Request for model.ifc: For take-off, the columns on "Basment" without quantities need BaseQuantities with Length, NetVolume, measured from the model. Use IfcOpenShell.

First a look at what the model holds.

```python
import ifcopenshell
import ifcopenshell.util.element
import ifcopenshell.util.unit

model = ifcopenshell.open("model.ifc")
print(model.schema)
for unit_type in ("LENGTHUNIT", "AREAUNIT", "VOLUMEUNIT"):
    print(unit_type, ifcopenshell.util.unit.calculate_unit_scale(model, unit_type))
storey = next(s for s in model.by_type("IfcBuildingStorey") if s.Name == "Basment")
columns = [e for e in ifcopenshell.util.element.get_decomposition(storey) if e.is_a("IfcColumn")]
for e in sorted(columns, key=lambda e: e.id()):
    print(e.id(), e.is_a(), e.Name, list(ifcopenshell.util.element.get_psets(e, qtos_only=True)), sep=" | ")
```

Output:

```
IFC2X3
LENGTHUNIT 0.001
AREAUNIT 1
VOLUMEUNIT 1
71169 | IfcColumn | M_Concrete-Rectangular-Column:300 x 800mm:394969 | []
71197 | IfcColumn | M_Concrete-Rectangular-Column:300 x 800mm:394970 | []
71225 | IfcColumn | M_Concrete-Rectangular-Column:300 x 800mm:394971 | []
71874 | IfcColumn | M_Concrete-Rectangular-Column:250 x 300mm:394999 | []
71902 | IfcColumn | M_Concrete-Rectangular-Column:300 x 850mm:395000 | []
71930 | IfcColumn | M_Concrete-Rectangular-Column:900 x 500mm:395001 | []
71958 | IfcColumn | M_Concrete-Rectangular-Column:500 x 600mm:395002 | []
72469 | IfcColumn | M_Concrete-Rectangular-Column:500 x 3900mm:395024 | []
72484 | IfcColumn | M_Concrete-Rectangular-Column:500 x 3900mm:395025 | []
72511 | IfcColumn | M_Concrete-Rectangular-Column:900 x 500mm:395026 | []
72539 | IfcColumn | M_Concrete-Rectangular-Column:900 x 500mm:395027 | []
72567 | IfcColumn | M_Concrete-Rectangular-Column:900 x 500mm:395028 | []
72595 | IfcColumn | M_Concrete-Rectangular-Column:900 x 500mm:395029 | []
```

```python
import ifcopenshell
import ifcopenshell.api.pset
import ifcopenshell.geom
import ifcopenshell.util.element
import ifcopenshell.util.shape
import ifcopenshell.util.unit

model = ifcopenshell.open("model.ifc")
unit_scale = ifcopenshell.util.unit.calculate_unit_scale(model)
volume_scale = ifcopenshell.util.unit.calculate_unit_scale(model, "VOLUMEUNIT")
settings = ifcopenshell.geom.settings()

storey = next(s for s in model.by_type("IfcBuildingStorey") if s.Name == "Basment")
columns = [e for e in ifcopenshell.util.element.get_decomposition(storey) if e.is_a("IfcColumn")]

for e in sorted(columns, key=lambda e: e.id()):
    if ifcopenshell.util.element.get_psets(e, qtos_only=True, should_inherit=False):
        continue
    # Geometry comes back in metres, in the element's own axes.
    shape = ifcopenshell.geom.create_shape(settings, e)
    values = {
        "Length": ifcopenshell.util.shape.get_z(shape.geometry) / unit_scale,
        "NetVolume": ifcopenshell.util.shape.get_volume(shape.geometry) / volume_scale,
    }
    qto = ifcopenshell.api.pset.add_qto(model, product=e, name="BaseQuantities")
    ifcopenshell.api.pset.edit_qto(model, qto=qto, properties=values)
    print(e.id(), {k: round(v, 3) for k, v in values.items()})

model.write("model-out.ifc")
```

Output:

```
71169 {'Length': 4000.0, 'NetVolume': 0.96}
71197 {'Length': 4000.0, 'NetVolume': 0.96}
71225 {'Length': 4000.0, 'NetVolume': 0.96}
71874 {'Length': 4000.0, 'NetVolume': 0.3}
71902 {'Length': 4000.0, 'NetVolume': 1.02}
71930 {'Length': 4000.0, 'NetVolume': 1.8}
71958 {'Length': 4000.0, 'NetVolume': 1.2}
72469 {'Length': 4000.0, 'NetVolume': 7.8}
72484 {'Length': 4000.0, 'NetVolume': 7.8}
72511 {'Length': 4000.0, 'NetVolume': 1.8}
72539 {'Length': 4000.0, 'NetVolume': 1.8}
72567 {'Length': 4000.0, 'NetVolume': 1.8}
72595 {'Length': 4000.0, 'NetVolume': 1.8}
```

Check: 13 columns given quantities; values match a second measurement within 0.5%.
